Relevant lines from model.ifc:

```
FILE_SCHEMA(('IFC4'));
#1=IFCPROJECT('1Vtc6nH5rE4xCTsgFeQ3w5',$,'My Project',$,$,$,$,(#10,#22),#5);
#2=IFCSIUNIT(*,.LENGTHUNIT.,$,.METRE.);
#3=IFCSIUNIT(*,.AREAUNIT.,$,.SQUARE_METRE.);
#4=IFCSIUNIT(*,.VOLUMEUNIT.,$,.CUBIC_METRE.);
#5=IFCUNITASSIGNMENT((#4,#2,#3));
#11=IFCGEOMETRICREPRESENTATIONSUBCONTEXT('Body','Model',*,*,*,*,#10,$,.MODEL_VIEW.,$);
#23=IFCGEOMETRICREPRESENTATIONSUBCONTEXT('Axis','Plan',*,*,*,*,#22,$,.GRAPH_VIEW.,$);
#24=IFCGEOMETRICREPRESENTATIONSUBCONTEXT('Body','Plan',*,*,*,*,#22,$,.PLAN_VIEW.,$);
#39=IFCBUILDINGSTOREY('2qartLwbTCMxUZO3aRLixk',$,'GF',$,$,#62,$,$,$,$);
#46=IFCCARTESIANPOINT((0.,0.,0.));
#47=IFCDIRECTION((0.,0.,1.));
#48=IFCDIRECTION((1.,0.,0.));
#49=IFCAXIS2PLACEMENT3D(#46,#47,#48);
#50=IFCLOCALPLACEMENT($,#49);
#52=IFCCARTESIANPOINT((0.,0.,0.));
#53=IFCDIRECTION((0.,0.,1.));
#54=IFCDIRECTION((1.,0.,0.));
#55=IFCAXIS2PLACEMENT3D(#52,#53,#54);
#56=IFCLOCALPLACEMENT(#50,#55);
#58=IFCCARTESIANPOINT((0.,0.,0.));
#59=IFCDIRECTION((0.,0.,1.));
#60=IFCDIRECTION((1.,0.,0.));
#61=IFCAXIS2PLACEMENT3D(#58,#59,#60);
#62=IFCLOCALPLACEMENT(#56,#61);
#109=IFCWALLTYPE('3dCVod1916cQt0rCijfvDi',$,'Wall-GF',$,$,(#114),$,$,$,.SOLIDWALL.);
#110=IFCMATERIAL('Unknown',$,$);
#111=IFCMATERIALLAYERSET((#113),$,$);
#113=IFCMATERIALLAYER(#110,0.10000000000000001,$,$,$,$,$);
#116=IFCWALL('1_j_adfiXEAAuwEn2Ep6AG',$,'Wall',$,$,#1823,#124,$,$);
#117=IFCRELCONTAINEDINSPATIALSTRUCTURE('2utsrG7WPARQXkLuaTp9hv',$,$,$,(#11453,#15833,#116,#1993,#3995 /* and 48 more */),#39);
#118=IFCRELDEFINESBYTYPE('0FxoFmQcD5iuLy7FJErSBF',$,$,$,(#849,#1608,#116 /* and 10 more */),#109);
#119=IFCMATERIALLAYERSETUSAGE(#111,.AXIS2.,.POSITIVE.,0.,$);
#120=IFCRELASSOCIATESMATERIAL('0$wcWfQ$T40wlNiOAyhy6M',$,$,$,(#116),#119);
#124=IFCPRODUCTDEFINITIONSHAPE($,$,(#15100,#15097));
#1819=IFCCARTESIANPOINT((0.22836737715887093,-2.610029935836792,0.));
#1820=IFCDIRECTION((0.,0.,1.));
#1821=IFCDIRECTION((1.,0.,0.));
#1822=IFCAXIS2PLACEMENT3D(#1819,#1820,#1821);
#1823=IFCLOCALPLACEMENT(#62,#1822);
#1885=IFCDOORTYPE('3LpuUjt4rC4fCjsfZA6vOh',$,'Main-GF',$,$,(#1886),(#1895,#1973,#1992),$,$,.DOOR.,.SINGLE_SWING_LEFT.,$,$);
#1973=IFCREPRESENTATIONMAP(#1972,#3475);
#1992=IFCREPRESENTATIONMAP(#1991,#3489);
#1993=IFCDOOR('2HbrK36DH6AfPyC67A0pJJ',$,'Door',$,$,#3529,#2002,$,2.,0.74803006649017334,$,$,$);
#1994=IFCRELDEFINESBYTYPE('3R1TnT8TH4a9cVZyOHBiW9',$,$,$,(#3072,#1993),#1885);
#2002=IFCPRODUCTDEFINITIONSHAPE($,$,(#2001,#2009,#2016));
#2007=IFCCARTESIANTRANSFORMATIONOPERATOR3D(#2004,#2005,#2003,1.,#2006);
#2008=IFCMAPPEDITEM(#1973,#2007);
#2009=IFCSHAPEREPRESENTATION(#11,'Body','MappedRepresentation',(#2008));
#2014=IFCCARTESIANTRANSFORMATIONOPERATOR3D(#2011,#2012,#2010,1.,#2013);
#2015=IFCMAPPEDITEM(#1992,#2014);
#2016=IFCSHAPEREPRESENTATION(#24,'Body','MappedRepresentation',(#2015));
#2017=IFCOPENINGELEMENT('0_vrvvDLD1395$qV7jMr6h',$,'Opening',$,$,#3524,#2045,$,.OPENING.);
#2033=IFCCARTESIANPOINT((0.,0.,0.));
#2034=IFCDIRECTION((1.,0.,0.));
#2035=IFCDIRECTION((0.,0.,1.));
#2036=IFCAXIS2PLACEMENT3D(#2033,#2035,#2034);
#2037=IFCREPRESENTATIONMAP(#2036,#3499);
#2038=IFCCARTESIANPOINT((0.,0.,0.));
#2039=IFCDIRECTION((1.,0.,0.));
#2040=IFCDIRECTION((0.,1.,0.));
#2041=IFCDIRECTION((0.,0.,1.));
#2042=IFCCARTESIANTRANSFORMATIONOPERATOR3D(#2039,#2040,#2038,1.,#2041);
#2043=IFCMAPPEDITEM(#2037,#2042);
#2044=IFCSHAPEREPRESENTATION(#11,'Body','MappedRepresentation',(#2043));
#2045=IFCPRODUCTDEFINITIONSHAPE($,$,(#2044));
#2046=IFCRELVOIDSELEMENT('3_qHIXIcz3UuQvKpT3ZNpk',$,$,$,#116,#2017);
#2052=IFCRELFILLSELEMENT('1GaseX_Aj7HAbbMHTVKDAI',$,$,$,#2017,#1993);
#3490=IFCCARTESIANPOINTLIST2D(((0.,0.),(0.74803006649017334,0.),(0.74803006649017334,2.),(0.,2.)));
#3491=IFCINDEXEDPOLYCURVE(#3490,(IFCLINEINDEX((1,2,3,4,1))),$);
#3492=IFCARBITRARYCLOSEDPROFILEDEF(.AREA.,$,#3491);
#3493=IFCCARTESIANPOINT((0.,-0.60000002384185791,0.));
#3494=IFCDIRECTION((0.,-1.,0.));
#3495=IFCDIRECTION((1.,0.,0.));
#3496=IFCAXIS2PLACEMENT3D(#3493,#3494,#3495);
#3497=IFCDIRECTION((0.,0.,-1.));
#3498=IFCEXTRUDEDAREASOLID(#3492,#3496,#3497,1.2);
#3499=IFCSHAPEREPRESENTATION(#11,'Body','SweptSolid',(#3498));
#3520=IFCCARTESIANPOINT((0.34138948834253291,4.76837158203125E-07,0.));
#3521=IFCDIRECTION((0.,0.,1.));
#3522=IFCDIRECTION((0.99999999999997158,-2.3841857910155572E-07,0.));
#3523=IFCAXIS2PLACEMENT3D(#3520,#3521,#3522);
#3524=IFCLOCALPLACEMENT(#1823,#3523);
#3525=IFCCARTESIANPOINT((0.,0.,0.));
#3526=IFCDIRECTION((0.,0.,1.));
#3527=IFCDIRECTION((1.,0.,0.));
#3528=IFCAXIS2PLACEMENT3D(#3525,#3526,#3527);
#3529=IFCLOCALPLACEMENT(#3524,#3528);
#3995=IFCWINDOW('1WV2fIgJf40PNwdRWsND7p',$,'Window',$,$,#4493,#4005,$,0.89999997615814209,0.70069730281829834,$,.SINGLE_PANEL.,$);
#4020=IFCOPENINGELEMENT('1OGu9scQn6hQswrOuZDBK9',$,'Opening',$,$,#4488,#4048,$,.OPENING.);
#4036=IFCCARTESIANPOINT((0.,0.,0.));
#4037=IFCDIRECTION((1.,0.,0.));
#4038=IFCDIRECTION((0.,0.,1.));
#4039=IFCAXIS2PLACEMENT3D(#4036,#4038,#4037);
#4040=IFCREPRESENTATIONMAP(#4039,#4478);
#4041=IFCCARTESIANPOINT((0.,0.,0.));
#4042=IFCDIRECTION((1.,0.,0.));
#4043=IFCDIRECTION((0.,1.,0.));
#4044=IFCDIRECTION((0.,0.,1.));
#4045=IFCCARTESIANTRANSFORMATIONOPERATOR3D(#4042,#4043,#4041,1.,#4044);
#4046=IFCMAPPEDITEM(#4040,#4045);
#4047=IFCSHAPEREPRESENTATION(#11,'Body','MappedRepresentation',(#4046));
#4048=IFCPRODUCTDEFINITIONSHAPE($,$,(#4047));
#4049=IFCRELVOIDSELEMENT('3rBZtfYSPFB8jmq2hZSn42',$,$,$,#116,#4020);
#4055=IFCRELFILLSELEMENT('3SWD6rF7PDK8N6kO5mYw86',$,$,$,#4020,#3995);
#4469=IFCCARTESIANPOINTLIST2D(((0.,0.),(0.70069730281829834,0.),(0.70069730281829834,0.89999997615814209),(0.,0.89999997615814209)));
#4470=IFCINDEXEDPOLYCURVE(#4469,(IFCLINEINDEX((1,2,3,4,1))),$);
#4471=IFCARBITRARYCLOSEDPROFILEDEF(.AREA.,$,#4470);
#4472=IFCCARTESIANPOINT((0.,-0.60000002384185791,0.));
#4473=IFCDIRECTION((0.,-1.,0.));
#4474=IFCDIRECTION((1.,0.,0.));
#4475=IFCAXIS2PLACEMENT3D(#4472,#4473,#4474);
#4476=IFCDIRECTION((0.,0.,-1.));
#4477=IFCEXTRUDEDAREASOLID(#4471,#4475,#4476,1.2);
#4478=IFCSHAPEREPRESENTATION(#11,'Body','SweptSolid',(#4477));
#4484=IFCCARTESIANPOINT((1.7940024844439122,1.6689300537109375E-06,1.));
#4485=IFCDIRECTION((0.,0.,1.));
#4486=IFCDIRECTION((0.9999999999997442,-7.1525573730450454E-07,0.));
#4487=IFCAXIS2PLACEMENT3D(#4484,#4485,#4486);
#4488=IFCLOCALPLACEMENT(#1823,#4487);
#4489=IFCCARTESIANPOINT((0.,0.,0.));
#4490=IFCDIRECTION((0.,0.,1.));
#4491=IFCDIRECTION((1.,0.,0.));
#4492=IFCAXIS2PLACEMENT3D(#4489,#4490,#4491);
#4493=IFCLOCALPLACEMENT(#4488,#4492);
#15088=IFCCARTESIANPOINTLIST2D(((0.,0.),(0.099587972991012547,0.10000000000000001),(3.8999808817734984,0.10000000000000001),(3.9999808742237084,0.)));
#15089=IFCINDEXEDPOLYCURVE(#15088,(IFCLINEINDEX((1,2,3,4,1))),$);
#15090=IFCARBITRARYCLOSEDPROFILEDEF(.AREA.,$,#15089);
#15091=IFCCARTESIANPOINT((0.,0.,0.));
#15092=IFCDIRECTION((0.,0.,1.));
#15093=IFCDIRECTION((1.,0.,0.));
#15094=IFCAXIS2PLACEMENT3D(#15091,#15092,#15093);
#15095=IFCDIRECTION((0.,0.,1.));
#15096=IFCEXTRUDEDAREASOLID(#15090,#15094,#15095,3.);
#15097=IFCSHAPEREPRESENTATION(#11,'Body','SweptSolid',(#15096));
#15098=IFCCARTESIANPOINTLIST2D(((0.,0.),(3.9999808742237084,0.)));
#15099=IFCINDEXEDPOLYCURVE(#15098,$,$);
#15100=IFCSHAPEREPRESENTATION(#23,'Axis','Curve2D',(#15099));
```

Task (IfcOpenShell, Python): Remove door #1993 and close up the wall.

```python
import ifcopenshell
import ifcopenshell.api.feature
import ifcopenshell.api.root
import ifcopenshell.geom
import ifcopenshell.util.shape

model = ifcopenshell.open("model.ifc")
settings = ifcopenshell.geom.settings()


def volume(element):
    """Net volume in cubic metres, openings subtracted."""
    shape = ifcopenshell.geom.create_shape(settings, element)
    return ifcopenshell.util.shape.get_volume(shape.geometry)


door = model.by_guid("2HbrK36DH6AfPyC67A0pJJ")
opening = door.FillsVoids[0].RelatingOpeningElement
wall = opening.VoidsElements[0].RelatingBuildingElement
before = volume(wall)

ifcopenshell.api.root.remove_product(model, product=door)
ifcopenshell.api.feature.remove_feature(model, feature=opening)

after = volume(wall)

print(f"wall volume {before:.3f} -> {after:.3f} m3")

model.write("model_updated.ifc")
```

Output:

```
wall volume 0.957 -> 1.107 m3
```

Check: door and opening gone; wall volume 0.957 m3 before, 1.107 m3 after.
